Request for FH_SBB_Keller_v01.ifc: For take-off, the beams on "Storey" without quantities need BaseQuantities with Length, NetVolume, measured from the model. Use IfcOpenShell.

First a look at what the model holds.

```python
import ifcopenshell
import ifcopenshell.util.element
import ifcopenshell.util.unit

model = ifcopenshell.open("FH_SBB_Keller_v01.ifc")
print(model.schema)
for unit_type in ("LENGTHUNIT", "AREAUNIT", "VOLUMEUNIT"):
    print(unit_type, ifcopenshell.util.unit.calculate_unit_scale(model, unit_type))
storey = next(s for s in model.by_type("IfcBuildingStorey") if s.Name == "Storey")
beams = [e for e in ifcopenshell.util.element.get_decomposition(storey) if e.is_a("IfcBeam")]
for e in sorted(beams, key=lambda e: e.id()):
    print(e.id(), e.is_a(), e.Name, list(ifcopenshell.util.element.get_psets(e, qtos_only=True)), sep=" | ")
```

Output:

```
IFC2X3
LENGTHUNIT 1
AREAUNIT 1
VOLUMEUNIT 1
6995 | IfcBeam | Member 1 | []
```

```python
import ifcopenshell
import ifcopenshell.api.pset
import ifcopenshell.geom
import ifcopenshell.util.element
import ifcopenshell.util.shape
import ifcopenshell.util.unit

model = ifcopenshell.open("FH_SBB_Keller_v01.ifc")
unit_scale = ifcopenshell.util.unit.calculate_unit_scale(model)
volume_scale = ifcopenshell.util.unit.calculate_unit_scale(model, "VOLUMEUNIT")
settings = ifcopenshell.geom.settings()

storey = next(s for s in model.by_type("IfcBuildingStorey") if s.Name == "Storey")
beams = [e for e in ifcopenshell.util.element.get_decomposition(storey) if e.is_a("IfcBeam")]

for e in sorted(beams, key=lambda e: e.id()):
    if ifcopenshell.util.element.get_psets(e, qtos_only=True, should_inherit=False):
        continue
    # Geometry comes back in metres, in the element's own axes.
    shape = ifcopenshell.geom.create_shape(settings, e)
    values = {
        "Length": ifcopenshell.util.shape.get_max_xyz(shape.geometry) / unit_scale,
        "NetVolume": ifcopenshell.util.shape.get_volume(shape.geometry) / volume_scale,
    }
    qto = ifcopenshell.api.pset.add_qto(model, product=e, name="BaseQuantities")
    ifcopenshell.api.pset.edit_qto(model, qto=qto, properties=values)
    print(e.id(), {k: round(v, 3) for k, v in values.items()})

model.write("FH_SBB_Keller_v01_v2.ifc")
```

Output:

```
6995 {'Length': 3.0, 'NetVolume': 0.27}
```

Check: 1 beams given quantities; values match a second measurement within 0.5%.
